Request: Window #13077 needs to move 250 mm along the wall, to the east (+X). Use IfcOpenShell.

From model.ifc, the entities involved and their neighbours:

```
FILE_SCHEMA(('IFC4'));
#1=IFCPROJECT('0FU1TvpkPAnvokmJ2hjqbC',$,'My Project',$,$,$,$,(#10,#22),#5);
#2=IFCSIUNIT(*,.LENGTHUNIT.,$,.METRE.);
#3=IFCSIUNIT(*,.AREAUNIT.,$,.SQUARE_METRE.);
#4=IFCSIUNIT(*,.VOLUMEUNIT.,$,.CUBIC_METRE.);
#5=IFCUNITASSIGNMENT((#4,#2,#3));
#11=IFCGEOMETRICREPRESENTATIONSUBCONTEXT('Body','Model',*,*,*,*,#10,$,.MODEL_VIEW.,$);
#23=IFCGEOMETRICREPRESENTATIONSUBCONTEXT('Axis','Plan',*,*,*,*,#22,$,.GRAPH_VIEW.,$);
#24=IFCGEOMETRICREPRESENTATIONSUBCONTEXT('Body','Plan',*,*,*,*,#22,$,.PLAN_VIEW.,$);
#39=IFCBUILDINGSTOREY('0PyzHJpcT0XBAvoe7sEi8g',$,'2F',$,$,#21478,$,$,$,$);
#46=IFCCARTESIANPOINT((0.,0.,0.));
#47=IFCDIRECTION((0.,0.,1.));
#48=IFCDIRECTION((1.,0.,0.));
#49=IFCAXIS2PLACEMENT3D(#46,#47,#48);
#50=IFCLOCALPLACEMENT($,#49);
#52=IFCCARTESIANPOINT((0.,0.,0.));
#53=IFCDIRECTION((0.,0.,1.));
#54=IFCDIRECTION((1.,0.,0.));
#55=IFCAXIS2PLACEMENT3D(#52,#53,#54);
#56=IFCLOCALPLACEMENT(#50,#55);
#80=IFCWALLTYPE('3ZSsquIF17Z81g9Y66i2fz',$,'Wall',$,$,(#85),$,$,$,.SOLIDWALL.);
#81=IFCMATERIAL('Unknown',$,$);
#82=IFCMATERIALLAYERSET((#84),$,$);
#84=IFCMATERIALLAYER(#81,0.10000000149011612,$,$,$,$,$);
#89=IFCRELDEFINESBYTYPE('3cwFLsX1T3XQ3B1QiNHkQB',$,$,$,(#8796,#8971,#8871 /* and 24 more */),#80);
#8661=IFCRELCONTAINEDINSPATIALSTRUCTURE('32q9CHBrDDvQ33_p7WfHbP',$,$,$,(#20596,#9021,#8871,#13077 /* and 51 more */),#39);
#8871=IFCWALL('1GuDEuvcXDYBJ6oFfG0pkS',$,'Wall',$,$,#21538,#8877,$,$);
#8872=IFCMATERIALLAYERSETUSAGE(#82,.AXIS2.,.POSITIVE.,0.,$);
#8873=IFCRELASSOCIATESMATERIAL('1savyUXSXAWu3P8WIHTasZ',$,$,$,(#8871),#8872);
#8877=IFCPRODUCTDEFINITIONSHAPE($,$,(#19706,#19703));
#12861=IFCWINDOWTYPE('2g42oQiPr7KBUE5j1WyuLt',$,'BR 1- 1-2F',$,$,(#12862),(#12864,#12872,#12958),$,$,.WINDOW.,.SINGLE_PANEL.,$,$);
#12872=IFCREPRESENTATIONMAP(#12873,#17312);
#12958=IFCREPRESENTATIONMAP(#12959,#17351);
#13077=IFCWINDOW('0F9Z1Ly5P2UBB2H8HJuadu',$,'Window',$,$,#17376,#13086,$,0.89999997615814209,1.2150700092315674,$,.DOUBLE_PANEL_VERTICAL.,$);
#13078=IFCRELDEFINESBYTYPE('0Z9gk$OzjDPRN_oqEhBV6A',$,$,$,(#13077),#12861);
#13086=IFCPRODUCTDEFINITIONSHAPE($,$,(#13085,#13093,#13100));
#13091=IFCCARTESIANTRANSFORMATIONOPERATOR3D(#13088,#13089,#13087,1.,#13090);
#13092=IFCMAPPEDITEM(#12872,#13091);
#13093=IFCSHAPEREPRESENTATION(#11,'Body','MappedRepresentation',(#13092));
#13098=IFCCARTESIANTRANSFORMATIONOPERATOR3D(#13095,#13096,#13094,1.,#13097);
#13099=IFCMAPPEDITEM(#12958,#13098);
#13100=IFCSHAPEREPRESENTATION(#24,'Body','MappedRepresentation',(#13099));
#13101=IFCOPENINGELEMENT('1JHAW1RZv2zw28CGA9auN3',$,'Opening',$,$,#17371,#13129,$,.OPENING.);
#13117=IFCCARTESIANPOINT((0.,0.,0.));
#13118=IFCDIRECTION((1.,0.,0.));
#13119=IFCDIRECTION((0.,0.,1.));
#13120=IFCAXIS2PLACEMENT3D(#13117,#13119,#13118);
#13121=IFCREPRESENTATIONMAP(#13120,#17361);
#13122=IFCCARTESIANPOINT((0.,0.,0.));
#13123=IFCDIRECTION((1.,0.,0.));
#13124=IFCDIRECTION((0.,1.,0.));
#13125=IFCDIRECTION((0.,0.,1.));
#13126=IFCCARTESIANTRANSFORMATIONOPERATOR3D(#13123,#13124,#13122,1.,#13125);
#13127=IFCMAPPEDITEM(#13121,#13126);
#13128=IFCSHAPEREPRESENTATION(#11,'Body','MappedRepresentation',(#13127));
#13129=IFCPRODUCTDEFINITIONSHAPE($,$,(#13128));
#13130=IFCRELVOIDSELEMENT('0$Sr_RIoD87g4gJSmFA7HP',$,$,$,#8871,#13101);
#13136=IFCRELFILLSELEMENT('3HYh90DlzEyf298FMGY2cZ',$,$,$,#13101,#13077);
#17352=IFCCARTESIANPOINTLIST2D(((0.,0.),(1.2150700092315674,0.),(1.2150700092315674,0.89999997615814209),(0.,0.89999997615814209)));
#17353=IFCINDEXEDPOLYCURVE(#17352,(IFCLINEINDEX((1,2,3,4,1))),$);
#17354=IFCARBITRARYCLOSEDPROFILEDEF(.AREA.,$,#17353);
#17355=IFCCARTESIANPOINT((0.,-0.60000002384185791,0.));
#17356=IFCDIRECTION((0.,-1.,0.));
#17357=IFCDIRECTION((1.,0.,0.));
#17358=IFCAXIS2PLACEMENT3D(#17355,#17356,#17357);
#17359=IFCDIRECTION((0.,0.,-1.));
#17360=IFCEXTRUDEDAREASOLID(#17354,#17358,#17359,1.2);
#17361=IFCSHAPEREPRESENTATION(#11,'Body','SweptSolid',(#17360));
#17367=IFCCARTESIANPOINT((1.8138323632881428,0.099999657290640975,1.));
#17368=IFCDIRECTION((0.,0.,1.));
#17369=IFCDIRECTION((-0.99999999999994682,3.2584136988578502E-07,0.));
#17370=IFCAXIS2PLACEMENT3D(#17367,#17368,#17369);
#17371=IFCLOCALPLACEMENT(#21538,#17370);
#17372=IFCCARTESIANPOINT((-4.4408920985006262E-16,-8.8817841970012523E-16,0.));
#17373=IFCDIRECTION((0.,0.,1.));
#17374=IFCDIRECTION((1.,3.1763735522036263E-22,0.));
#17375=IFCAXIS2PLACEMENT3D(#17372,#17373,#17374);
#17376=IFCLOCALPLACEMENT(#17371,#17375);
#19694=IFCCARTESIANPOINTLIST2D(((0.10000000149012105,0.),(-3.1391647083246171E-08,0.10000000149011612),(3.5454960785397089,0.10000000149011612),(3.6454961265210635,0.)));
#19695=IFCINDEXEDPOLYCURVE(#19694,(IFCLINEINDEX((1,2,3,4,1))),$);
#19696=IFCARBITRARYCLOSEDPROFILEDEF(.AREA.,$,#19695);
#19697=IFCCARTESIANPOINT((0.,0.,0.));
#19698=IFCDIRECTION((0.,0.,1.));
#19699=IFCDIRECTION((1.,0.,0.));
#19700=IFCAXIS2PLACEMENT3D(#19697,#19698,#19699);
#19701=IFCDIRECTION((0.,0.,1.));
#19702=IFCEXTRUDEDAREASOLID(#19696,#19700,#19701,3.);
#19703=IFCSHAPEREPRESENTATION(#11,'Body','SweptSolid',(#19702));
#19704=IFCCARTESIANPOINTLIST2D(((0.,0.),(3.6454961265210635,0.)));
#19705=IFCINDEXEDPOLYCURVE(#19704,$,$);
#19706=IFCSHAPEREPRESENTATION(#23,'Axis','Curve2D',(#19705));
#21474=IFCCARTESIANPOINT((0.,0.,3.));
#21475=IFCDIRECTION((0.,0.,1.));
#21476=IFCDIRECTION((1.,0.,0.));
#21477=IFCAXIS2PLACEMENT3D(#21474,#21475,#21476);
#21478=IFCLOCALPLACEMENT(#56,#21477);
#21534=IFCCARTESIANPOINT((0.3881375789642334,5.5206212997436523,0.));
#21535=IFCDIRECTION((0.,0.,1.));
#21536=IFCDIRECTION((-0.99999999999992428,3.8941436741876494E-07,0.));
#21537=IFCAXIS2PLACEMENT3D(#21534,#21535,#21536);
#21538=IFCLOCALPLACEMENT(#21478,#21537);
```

```python
import ifcopenshell
import ifcopenshell.api.geometry
import ifcopenshell.util.placement
import ifcopenshell.util.unit

model = ifcopenshell.open("model.ifc")
unit_scale = ifcopenshell.util.unit.calculate_unit_scale(model)

window = model.by_guid("0F9Z1Ly5P2UBB2H8HJuadu")
opening = window.FillsVoids[0].RelatingOpeningElement
wall = opening.VoidsElements[0].RelatingBuildingElement

wall_matrix = ifcopenshell.util.placement.get_local_placement(wall.ObjectPlacement)
shift = wall_matrix[:3, 0] * -0.25 / unit_scale
before = ifcopenshell.util.placement.get_local_placement(window.ObjectPlacement)[:3, 3].copy()

# The window is placed relative to its opening, so it follows when the opening moves.
matrix = ifcopenshell.util.placement.get_local_placement(opening.ObjectPlacement)
matrix[:3, 3] += shift
ifcopenshell.api.geometry.edit_object_placement(
    model, product=opening, matrix=matrix, is_si=False, should_transform_children=True
)

after = ifcopenshell.util.placement.get_local_placement(window.ObjectPlacement)[:3, 3]
print("window moved by", (after - before).round(3) + 0.0)

model.write("model_edited.ifc")
```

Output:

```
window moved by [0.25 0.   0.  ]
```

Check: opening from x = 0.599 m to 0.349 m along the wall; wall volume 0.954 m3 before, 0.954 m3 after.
